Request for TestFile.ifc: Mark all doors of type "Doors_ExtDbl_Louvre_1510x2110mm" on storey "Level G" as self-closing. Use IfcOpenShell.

First a look at what the model holds.

```python
import ifcopenshell
import ifcopenshell.util.element

model = ifcopenshell.open("TestFile.ifc")
print(model.schema)
storey = next(s for s in model.by_type("IfcBuildingStorey") if s.Name == "Level G")
doors = [e for e in ifcopenshell.util.element.get_decomposition(storey) if e.is_a("IfcDoor")]
seen = {}
for e in doors:
    element_type = ifcopenshell.util.element.get_type(e)
    key = (element_type.Name if element_type != e and element_type else None, ifcopenshell.util.element.get_pset(e, "Pset_DoorCommon", "SelfClosing"))
    seen[key] = seen.get(key, 0) + 1
for (name, value), count in sorted(seen.items(), key=str):
    print(count, "x", name, "|", value)
```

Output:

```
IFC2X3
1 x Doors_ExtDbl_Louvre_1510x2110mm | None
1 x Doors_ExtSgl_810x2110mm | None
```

```python
import ifcopenshell
import ifcopenshell.api.pset
import ifcopenshell.util.element

model = ifcopenshell.open("TestFile.ifc")

storey = next(s for s in model.by_type("IfcBuildingStorey") if s.Name == "Level G")
doors = [e for e in ifcopenshell.util.element.get_decomposition(storey) if e.is_a("IfcDoor")]

count = 0
for e in doors:
    element_type = ifcopenshell.util.element.get_type(e)
    if element_type in (None, e) or element_type.Name != "Doors_ExtDbl_Louvre_1510x2110mm":
        continue
    # add_pset returns the element's existing set when there is one.
    pset = ifcopenshell.api.pset.add_pset(model, product=e, name="Pset_DoorCommon")
    ifcopenshell.api.pset.edit_pset(model, pset=pset, properties={"SelfClosing": True})
    count += 1

print(count, "doors updated")

model.write("TestFile-out.ifc")
```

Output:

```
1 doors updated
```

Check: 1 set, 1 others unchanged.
